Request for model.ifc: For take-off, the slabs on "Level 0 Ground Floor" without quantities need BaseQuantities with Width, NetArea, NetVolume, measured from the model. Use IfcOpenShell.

First a look at what the model holds.

```python
import ifcopenshell
import ifcopenshell.util.element
import ifcopenshell.util.unit

model = ifcopenshell.open("model.ifc")
print(model.schema)
for unit_type in ("LENGTHUNIT", "AREAUNIT", "VOLUMEUNIT"):
    print(unit_type, ifcopenshell.util.unit.calculate_unit_scale(model, unit_type))
storey = next(s for s in model.by_type("IfcBuildingStorey") if s.Name == "Level 0 Ground Floor")
slabs = [e for e in ifcopenshell.util.element.get_decomposition(storey) if e.is_a("IfcSlab")]
for e in sorted(slabs, key=lambda e: e.id()):
    print(e.id(), e.is_a(), e.Name, list(ifcopenshell.util.element.get_psets(e, qtos_only=True)), sep=" | ")
```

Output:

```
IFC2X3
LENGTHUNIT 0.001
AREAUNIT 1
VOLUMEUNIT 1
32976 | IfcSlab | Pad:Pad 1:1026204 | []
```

```python
import ifcopenshell
import ifcopenshell.api.pset
import ifcopenshell.geom
import ifcopenshell.util.element
import ifcopenshell.util.shape
import ifcopenshell.util.unit

model = ifcopenshell.open("model.ifc")
unit_scale = ifcopenshell.util.unit.calculate_unit_scale(model)
area_scale = ifcopenshell.util.unit.calculate_unit_scale(model, "AREAUNIT")
volume_scale = ifcopenshell.util.unit.calculate_unit_scale(model, "VOLUMEUNIT")
settings = ifcopenshell.geom.settings()

storey = next(s for s in model.by_type("IfcBuildingStorey") if s.Name == "Level 0 Ground Floor")
slabs = [e for e in ifcopenshell.util.element.get_decomposition(storey) if e.is_a("IfcSlab")]

for e in sorted(slabs, key=lambda e: e.id()):
    if ifcopenshell.util.element.get_psets(e, qtos_only=True, should_inherit=False):
        continue
    # Geometry comes back in metres, in the element's own axes.
    shape = ifcopenshell.geom.create_shape(settings, e)
    values = {
        "Width": ifcopenshell.util.shape.get_z(shape.geometry) / unit_scale,
        "NetArea": ifcopenshell.util.shape.get_footprint_area(shape.geometry) / area_scale,
        "NetVolume": ifcopenshell.util.shape.get_volume(shape.geometry) / volume_scale,
    }
    qto = ifcopenshell.api.pset.add_qto(model, product=e, name="BaseQuantities")
    ifcopenshell.api.pset.edit_qto(model, qto=qto, properties=values)
    print(e.id(), {k: round(v, 3) for k, v in values.items()})

model.write("model_edited.ifc")
```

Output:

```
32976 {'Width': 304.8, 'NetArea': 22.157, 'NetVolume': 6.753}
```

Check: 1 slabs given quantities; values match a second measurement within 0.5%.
